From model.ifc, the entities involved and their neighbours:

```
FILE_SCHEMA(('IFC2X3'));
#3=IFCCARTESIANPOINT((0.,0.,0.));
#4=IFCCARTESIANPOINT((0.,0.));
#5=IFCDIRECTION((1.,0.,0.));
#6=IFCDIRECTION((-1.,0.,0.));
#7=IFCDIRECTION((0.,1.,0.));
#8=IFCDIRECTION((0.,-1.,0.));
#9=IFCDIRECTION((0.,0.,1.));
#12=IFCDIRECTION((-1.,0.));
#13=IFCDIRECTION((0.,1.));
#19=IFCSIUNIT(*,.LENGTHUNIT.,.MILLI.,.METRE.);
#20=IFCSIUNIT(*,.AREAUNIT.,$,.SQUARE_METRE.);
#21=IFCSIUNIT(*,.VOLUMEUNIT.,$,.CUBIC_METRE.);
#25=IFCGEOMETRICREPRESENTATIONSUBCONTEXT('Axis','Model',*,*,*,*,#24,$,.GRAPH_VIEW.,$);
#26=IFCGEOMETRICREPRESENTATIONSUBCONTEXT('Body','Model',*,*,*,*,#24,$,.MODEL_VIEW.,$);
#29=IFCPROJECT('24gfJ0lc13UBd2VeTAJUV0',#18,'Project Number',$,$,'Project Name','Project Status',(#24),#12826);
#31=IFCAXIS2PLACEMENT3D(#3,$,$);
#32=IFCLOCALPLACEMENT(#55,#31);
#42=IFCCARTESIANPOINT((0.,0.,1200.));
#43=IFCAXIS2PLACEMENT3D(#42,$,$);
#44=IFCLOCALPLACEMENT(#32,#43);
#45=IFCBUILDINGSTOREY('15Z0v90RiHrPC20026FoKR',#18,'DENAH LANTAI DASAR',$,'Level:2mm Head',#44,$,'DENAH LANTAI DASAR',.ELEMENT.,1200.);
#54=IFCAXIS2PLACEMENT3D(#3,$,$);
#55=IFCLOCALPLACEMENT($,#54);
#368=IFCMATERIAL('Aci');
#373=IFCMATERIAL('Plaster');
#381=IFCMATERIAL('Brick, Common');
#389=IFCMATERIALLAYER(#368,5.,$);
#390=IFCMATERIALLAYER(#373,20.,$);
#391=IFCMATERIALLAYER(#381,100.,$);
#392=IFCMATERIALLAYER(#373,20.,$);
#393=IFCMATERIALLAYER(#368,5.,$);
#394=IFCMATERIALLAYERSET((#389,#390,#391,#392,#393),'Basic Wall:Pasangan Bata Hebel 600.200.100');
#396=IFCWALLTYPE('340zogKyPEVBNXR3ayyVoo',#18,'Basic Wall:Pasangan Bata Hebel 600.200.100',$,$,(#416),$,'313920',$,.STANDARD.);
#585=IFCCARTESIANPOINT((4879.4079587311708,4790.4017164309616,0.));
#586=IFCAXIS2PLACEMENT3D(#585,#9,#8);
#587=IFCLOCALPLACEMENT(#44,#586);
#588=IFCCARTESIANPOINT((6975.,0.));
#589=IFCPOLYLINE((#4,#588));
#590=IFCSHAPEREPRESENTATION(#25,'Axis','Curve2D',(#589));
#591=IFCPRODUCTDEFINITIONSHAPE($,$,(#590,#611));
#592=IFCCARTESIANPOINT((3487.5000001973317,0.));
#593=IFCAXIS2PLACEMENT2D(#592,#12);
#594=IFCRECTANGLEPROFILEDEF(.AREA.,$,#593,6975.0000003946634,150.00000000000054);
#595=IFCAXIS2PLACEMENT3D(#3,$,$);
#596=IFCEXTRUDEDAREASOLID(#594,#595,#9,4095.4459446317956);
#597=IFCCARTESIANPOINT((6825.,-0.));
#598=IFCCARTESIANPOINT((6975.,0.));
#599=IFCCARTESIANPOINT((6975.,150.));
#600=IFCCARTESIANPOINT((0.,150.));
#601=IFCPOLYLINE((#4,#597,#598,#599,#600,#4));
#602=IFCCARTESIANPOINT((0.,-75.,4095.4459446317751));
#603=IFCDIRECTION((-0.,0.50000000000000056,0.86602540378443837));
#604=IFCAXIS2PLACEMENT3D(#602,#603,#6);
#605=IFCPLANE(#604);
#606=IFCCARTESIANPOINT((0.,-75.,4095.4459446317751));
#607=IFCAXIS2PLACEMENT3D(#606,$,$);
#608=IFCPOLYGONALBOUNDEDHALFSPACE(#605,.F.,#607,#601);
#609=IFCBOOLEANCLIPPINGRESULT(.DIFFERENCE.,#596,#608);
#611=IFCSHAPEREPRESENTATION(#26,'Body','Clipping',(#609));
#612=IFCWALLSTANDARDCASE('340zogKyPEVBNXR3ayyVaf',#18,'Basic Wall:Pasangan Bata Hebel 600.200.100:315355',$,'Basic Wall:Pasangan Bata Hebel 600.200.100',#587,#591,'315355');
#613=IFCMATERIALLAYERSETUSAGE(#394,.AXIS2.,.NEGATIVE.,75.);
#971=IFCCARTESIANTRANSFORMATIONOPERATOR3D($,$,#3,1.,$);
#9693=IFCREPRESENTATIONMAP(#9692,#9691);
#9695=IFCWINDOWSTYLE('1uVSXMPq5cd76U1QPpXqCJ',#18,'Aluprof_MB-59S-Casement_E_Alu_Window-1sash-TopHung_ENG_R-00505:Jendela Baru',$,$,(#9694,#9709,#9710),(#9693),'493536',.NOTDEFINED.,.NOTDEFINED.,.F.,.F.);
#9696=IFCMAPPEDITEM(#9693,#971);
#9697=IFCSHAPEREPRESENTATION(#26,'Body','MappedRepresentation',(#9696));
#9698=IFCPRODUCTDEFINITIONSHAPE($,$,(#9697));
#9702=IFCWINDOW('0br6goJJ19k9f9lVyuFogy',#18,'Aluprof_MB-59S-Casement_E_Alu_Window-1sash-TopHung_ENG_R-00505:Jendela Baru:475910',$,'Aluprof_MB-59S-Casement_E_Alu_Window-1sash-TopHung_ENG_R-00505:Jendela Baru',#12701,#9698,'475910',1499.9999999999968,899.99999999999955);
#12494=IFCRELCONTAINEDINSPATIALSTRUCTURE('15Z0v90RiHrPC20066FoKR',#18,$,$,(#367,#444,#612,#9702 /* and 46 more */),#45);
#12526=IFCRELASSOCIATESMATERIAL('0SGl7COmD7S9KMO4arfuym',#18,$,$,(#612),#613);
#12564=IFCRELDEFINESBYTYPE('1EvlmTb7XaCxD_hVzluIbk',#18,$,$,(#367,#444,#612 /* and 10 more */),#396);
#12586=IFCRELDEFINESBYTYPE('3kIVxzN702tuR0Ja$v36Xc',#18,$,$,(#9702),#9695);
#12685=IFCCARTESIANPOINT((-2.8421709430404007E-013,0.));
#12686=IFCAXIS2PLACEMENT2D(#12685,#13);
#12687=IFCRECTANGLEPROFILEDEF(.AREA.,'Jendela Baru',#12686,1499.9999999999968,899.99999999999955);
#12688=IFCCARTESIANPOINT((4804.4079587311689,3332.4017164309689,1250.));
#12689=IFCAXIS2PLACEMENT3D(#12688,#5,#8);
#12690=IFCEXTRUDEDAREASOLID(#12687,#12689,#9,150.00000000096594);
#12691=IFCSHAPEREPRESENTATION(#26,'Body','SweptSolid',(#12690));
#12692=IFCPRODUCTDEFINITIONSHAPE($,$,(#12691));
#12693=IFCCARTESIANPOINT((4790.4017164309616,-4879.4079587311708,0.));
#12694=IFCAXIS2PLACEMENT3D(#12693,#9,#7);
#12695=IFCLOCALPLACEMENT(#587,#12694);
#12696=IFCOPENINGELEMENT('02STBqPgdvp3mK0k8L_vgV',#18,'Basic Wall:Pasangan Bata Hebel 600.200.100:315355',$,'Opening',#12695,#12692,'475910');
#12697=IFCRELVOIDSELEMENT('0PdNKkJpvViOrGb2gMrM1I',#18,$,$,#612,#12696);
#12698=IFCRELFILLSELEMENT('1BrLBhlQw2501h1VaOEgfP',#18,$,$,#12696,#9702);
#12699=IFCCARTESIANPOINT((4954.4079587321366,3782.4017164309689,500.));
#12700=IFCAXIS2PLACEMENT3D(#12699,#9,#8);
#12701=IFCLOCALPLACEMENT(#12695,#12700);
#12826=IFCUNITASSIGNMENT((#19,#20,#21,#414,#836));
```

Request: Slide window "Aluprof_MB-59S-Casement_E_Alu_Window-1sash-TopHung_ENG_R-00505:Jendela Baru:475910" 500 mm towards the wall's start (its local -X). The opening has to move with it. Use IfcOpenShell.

```python
import ifcopenshell
import ifcopenshell.api.geometry
import ifcopenshell.util.placement
import ifcopenshell.util.unit

model = ifcopenshell.open("model.ifc")
unit_scale = ifcopenshell.util.unit.calculate_unit_scale(model)

window = model.by_guid("0br6goJJ19k9f9lVyuFogy")
opening = window.FillsVoids[0].RelatingOpeningElement
wall = opening.VoidsElements[0].RelatingBuildingElement

wall_matrix = ifcopenshell.util.placement.get_local_placement(wall.ObjectPlacement)
shift = wall_matrix[:3, 0] * -0.5 / unit_scale
before = ifcopenshell.util.placement.get_local_placement(window.ObjectPlacement)[:3, 3].copy()

# The window is placed relative to its opening, so it follows when the opening moves.
matrix = ifcopenshell.util.placement.get_local_placement(opening.ObjectPlacement)
matrix[:3, 3] += shift
ifcopenshell.api.geometry.edit_object_placement(
    model, product=opening, matrix=matrix, is_si=False, should_transform_children=True
)

after = ifcopenshell.util.placement.get_local_placement(window.ObjectPlacement)[:3, 3]
print("window moved by", (after - before).round(3) + 0.0)

model.write("model_updated.ifc")
```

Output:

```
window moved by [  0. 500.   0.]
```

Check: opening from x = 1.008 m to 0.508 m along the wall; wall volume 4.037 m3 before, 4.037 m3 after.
